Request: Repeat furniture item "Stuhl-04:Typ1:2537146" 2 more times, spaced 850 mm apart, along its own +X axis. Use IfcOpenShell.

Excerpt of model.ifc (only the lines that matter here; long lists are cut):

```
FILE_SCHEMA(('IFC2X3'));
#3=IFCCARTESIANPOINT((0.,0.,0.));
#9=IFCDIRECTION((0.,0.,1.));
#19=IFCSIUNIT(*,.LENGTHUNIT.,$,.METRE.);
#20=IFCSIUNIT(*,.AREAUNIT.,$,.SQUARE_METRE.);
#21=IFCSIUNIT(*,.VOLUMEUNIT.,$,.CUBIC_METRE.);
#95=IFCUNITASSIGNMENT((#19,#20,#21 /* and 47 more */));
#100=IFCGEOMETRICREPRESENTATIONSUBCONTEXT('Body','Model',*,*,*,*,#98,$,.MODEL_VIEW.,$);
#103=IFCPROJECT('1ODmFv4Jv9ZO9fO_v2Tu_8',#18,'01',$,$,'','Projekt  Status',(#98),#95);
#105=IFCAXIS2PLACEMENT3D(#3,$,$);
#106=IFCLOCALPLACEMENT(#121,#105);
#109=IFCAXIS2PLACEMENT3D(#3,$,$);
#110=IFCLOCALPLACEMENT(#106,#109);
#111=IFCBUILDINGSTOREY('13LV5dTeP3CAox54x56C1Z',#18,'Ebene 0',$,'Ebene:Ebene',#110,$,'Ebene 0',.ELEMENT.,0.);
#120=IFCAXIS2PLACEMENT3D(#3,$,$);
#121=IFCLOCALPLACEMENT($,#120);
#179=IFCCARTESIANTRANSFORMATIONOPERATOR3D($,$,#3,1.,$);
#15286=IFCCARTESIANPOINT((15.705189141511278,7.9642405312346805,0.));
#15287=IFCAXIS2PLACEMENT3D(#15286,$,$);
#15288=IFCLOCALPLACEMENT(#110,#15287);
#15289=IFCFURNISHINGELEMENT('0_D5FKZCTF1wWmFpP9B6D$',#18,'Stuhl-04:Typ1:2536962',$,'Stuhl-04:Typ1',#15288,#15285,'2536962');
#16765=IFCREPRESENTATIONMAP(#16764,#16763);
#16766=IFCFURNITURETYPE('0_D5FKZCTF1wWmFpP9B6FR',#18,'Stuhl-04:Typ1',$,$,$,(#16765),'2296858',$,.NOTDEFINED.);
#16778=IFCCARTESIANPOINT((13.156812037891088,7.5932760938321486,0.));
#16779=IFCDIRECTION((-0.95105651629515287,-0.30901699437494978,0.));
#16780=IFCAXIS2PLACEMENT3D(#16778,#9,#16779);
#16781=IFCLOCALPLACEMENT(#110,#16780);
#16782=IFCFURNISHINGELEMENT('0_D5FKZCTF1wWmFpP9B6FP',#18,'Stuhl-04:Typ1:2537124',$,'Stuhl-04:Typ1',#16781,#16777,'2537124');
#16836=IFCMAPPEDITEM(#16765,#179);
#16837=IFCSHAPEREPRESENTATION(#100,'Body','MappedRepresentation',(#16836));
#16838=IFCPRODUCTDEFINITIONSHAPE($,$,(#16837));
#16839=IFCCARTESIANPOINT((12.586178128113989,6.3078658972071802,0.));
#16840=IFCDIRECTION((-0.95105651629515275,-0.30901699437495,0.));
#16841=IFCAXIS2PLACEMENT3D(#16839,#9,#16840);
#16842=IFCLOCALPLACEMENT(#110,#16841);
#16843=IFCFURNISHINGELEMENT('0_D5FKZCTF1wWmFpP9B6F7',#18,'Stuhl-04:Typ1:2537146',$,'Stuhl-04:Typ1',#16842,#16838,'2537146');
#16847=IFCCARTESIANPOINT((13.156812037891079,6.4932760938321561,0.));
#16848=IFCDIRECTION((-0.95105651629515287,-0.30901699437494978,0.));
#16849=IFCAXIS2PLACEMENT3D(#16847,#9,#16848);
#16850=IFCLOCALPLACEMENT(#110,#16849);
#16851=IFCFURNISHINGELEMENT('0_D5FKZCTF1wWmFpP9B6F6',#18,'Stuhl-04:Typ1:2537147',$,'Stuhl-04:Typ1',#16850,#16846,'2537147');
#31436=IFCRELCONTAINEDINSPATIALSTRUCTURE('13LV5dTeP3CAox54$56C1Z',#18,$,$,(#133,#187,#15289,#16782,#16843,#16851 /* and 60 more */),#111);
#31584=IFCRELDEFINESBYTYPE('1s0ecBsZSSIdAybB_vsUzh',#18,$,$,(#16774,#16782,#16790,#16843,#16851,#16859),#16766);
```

```python
import ifcopenshell
import ifcopenshell.api.geometry
import ifcopenshell.api.root
import ifcopenshell.util.element
import ifcopenshell.util.placement
import ifcopenshell.util.unit

model = ifcopenshell.open("model.ifc")
unit_scale = ifcopenshell.util.unit.calculate_unit_scale(model)

source = model.by_guid("0_D5FKZCTF1wWmFpP9B6F7")
base = ifcopenshell.util.placement.get_local_placement(source.ObjectPlacement)
step = base[:3, 0] * 0.85 / unit_scale

for i in range(1, 3):
    copy = ifcopenshell.api.root.copy_class(model, product=source)
    copy.Representation = ifcopenshell.util.element.copy_deep(
        model, source.Representation, exclude=["IfcGeometricRepresentationContext", "IfcRepresentationMap"]
    )
    copy.Name = "Stuhl-04:Typ1"
    copy.Tag = None
    matrix = base.copy()
    matrix[:3, 3] += i * step
    print("added at", matrix[:3, 3].round(3) + 0.0)
    ifcopenshell.api.geometry.edit_object_placement(model, product=copy, matrix=matrix, is_si=False)

model.write("model_updated.ifc")
```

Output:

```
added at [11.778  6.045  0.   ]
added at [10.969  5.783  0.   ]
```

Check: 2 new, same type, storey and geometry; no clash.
